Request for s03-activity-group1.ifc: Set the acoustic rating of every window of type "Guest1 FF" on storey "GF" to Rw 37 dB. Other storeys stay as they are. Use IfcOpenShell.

First a look at what the model holds.

```python
import ifcopenshell
import ifcopenshell.util.element

model = ifcopenshell.open("s03-activity-group1.ifc")
print(model.schema)
storey = next(s for s in model.by_type("IfcBuildingStorey") if s.Name == "GF")
windows = [e for e in ifcopenshell.util.element.get_decomposition(storey) if e.is_a("IfcWindow")]
seen = {}
for e in windows:
    element_type = ifcopenshell.util.element.get_type(e)
    key = (element_type.Name if element_type != e and element_type else None, ifcopenshell.util.element.get_pset(e, "Pset_WindowCommon", "AcousticRating"))
    seen[key] = seen.get(key, 0) + 1
for (name, value), count in sorted(seen.items(), key=str):
    print(count, "x", name, "|", value)
```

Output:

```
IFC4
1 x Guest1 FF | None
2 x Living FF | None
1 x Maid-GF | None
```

```python
import ifcopenshell
import ifcopenshell.api.pset
import ifcopenshell.util.element

model = ifcopenshell.open("s03-activity-group1.ifc")

storey = next(s for s in model.by_type("IfcBuildingStorey") if s.Name == "GF")
windows = [e for e in ifcopenshell.util.element.get_decomposition(storey) if e.is_a("IfcWindow")]

count = 0
for e in windows:
    element_type = ifcopenshell.util.element.get_type(e)
    if element_type in (None, e) or element_type.Name != "Guest1 FF":
        continue
    # add_pset returns the element's existing set when there is one.
    pset = ifcopenshell.api.pset.add_pset(model, product=e, name="Pset_WindowCommon")
    ifcopenshell.api.pset.edit_pset(model, pset=pset, properties={"AcousticRating": "Rw 37 dB"})
    count += 1

print(count, "windows updated")

model.write("s03-activity-group1_rev.ifc")
```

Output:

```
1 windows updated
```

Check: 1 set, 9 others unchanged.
